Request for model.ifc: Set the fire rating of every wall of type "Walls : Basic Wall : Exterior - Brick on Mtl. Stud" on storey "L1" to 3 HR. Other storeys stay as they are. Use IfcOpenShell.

First a look at what the model holds.

```python
import ifcopenshell
import ifcopenshell.util.element

model = ifcopenshell.open("model.ifc")
print(model.schema)
storey = next(s for s in model.by_type("IfcBuildingStorey") if s.Name == "L1")
walls = [e for e in ifcopenshell.util.element.get_decomposition(storey) if e.is_a("IfcWall")]
seen = {}
for e in walls:
    element_type = ifcopenshell.util.element.get_type(e)
    key = (element_type.Name if element_type != e and element_type else None, ifcopenshell.util.element.get_pset(e, "Pset_WallCommon", "FireRating"))
    seen[key] = seen.get(key, 0) + 1
for (name, value), count in sorted(seen.items(), key=str):
    print(count, "x", name, "|", value)
```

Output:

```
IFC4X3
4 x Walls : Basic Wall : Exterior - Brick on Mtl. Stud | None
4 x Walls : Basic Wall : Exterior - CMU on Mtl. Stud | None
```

```python
import ifcopenshell
import ifcopenshell.api.pset
import ifcopenshell.util.element

model = ifcopenshell.open("model.ifc")

storey = next(s for s in model.by_type("IfcBuildingStorey") if s.Name == "L1")
walls = [e for e in ifcopenshell.util.element.get_decomposition(storey) if e.is_a("IfcWall")]

count = 0
for e in walls:
    element_type = ifcopenshell.util.element.get_type(e)
    if element_type in (None, e) or element_type.Name != "Walls : Basic Wall : Exterior - Brick on Mtl. Stud":
        continue
    # add_pset returns the element's existing set when there is one.
    pset = ifcopenshell.api.pset.add_pset(model, product=e, name="Pset_WallCommon")
    ifcopenshell.api.pset.edit_pset(model, pset=pset, properties={"FireRating": "3 HR"})
    count += 1

print(count, "walls updated")

model.write("model_edited.ifc")
```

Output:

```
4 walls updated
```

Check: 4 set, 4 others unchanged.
